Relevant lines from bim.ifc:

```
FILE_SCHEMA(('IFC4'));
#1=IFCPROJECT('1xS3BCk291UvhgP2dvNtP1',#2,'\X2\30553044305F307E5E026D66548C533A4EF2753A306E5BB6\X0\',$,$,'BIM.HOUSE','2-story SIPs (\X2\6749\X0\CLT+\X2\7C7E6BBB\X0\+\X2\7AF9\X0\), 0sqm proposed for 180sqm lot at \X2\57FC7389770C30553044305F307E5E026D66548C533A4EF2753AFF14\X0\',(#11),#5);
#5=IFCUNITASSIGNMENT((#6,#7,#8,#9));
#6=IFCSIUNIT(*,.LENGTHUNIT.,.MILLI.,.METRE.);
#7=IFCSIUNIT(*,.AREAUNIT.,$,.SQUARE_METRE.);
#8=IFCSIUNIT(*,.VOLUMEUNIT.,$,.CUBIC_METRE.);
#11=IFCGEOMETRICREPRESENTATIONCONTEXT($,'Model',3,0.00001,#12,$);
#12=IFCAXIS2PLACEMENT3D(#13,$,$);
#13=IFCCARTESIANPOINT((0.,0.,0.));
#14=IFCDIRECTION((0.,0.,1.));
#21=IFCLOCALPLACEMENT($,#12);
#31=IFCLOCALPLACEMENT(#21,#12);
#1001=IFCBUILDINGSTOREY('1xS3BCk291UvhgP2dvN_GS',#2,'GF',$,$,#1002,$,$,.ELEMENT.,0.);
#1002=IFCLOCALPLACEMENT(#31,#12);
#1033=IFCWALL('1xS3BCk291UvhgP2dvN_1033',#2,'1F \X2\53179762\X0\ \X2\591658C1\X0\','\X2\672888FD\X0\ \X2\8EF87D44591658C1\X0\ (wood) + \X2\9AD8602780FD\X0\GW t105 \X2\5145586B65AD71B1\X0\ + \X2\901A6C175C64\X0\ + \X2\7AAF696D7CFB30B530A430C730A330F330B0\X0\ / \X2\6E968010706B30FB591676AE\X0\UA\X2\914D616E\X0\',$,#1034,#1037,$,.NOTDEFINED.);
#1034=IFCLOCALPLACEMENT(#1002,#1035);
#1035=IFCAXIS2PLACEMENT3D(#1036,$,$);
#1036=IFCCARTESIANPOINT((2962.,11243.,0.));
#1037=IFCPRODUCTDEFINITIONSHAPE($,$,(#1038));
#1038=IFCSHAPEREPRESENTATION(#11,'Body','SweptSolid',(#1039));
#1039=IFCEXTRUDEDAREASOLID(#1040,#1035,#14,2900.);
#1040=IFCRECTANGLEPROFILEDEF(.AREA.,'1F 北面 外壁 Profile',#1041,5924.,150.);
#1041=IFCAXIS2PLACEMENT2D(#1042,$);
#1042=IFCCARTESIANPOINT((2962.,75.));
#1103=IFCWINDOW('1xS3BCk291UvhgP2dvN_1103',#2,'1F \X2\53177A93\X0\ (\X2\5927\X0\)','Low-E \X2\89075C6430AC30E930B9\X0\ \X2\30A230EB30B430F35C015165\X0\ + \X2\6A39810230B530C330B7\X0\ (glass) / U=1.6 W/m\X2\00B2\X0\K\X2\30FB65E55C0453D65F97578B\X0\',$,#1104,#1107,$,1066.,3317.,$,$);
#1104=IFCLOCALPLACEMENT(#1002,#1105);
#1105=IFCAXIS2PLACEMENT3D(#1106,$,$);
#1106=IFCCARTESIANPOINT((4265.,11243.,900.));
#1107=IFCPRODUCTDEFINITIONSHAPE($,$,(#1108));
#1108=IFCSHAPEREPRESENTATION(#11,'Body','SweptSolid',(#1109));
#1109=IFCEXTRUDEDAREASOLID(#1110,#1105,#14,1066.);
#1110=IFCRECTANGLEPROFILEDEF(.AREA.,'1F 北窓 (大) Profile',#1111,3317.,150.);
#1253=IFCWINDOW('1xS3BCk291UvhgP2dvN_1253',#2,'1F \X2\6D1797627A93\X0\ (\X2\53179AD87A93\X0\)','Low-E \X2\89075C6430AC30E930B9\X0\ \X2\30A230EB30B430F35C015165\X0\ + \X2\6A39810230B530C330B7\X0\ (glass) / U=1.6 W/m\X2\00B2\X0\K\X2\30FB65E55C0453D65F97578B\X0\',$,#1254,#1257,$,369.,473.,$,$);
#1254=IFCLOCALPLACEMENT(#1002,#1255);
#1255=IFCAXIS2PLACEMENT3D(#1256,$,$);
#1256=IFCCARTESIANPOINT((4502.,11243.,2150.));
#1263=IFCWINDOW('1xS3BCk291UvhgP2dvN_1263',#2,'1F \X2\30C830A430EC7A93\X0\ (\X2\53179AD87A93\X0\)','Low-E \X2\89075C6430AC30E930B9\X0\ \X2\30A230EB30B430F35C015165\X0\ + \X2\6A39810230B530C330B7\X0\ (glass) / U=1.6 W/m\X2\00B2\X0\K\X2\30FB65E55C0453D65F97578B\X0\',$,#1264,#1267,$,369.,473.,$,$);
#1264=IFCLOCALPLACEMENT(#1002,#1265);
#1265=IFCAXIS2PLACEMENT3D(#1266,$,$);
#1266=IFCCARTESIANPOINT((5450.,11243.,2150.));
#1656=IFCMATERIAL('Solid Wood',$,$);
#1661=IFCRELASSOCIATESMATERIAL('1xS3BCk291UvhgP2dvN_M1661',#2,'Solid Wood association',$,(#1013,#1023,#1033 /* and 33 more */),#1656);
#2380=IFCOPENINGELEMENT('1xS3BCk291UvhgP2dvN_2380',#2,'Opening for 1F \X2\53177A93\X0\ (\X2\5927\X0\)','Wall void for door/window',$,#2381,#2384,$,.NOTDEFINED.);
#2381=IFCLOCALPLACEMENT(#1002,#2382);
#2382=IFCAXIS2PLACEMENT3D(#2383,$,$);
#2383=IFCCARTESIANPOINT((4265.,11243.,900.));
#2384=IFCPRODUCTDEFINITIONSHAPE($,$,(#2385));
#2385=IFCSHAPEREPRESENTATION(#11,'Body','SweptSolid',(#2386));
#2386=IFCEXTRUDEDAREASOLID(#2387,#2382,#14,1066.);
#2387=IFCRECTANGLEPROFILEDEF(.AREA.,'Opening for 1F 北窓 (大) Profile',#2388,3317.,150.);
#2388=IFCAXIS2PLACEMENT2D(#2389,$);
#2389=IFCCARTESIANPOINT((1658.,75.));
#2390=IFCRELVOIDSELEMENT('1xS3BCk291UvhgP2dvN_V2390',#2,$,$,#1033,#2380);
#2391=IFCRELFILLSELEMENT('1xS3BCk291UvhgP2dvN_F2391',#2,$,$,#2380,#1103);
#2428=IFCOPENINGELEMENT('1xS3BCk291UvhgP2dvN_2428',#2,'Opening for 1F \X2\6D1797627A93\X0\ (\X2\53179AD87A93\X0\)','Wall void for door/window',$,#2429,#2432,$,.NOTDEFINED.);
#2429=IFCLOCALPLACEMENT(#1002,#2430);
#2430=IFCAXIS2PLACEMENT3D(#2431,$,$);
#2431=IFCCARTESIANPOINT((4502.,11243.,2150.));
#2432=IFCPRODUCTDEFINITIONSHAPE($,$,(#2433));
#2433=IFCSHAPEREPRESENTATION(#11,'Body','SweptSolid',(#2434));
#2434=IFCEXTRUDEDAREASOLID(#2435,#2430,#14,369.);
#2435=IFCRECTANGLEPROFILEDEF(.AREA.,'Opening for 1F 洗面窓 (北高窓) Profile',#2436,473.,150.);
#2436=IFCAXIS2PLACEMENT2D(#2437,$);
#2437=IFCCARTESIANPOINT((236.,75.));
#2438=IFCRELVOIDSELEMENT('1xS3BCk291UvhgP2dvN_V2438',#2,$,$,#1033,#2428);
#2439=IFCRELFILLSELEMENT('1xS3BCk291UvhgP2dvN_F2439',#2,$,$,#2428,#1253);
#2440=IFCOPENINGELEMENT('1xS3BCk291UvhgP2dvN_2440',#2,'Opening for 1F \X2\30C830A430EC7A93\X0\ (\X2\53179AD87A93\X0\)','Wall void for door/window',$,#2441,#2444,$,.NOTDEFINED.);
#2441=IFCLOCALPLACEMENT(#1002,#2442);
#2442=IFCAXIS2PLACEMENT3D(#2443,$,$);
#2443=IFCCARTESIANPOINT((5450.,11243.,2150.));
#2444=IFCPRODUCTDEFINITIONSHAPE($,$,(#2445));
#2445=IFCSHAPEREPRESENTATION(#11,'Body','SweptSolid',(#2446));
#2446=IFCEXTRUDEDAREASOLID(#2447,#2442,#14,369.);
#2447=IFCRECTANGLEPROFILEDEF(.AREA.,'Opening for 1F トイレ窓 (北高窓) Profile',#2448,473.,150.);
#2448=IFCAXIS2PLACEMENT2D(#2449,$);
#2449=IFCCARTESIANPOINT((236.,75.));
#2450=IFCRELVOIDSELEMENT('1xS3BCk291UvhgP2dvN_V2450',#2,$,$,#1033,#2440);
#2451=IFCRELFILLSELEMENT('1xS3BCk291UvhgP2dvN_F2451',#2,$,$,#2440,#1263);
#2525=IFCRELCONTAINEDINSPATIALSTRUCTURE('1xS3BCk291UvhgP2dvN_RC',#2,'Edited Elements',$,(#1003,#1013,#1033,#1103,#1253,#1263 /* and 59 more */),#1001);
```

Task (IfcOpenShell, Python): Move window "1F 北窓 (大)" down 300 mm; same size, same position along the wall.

```python
import numpy as np
import ifcopenshell
import ifcopenshell.api.geometry
import ifcopenshell.util.placement
import ifcopenshell.util.unit

model = ifcopenshell.open("bim.ifc")
unit_scale = ifcopenshell.util.unit.calculate_unit_scale(model)

window = model.by_id(1103)
opening = window.FillsVoids[0].RelatingOpeningElement
dz = -300.0

shift = np.array([0.0, 0.0, dz])
# The window is not placed relative to its opening, so move both.
for product in (opening, window):
    matrix = ifcopenshell.util.placement.get_local_placement(product.ObjectPlacement)
    matrix[:3, 3] += shift
    ifcopenshell.api.geometry.edit_object_placement(model, product=product, matrix=matrix, is_si=False)

print(f"moved by {dz * unit_scale:+.3f} m")

model.write("bim_edited.ifc")
```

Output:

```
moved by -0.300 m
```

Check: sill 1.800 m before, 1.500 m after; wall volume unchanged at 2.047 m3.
